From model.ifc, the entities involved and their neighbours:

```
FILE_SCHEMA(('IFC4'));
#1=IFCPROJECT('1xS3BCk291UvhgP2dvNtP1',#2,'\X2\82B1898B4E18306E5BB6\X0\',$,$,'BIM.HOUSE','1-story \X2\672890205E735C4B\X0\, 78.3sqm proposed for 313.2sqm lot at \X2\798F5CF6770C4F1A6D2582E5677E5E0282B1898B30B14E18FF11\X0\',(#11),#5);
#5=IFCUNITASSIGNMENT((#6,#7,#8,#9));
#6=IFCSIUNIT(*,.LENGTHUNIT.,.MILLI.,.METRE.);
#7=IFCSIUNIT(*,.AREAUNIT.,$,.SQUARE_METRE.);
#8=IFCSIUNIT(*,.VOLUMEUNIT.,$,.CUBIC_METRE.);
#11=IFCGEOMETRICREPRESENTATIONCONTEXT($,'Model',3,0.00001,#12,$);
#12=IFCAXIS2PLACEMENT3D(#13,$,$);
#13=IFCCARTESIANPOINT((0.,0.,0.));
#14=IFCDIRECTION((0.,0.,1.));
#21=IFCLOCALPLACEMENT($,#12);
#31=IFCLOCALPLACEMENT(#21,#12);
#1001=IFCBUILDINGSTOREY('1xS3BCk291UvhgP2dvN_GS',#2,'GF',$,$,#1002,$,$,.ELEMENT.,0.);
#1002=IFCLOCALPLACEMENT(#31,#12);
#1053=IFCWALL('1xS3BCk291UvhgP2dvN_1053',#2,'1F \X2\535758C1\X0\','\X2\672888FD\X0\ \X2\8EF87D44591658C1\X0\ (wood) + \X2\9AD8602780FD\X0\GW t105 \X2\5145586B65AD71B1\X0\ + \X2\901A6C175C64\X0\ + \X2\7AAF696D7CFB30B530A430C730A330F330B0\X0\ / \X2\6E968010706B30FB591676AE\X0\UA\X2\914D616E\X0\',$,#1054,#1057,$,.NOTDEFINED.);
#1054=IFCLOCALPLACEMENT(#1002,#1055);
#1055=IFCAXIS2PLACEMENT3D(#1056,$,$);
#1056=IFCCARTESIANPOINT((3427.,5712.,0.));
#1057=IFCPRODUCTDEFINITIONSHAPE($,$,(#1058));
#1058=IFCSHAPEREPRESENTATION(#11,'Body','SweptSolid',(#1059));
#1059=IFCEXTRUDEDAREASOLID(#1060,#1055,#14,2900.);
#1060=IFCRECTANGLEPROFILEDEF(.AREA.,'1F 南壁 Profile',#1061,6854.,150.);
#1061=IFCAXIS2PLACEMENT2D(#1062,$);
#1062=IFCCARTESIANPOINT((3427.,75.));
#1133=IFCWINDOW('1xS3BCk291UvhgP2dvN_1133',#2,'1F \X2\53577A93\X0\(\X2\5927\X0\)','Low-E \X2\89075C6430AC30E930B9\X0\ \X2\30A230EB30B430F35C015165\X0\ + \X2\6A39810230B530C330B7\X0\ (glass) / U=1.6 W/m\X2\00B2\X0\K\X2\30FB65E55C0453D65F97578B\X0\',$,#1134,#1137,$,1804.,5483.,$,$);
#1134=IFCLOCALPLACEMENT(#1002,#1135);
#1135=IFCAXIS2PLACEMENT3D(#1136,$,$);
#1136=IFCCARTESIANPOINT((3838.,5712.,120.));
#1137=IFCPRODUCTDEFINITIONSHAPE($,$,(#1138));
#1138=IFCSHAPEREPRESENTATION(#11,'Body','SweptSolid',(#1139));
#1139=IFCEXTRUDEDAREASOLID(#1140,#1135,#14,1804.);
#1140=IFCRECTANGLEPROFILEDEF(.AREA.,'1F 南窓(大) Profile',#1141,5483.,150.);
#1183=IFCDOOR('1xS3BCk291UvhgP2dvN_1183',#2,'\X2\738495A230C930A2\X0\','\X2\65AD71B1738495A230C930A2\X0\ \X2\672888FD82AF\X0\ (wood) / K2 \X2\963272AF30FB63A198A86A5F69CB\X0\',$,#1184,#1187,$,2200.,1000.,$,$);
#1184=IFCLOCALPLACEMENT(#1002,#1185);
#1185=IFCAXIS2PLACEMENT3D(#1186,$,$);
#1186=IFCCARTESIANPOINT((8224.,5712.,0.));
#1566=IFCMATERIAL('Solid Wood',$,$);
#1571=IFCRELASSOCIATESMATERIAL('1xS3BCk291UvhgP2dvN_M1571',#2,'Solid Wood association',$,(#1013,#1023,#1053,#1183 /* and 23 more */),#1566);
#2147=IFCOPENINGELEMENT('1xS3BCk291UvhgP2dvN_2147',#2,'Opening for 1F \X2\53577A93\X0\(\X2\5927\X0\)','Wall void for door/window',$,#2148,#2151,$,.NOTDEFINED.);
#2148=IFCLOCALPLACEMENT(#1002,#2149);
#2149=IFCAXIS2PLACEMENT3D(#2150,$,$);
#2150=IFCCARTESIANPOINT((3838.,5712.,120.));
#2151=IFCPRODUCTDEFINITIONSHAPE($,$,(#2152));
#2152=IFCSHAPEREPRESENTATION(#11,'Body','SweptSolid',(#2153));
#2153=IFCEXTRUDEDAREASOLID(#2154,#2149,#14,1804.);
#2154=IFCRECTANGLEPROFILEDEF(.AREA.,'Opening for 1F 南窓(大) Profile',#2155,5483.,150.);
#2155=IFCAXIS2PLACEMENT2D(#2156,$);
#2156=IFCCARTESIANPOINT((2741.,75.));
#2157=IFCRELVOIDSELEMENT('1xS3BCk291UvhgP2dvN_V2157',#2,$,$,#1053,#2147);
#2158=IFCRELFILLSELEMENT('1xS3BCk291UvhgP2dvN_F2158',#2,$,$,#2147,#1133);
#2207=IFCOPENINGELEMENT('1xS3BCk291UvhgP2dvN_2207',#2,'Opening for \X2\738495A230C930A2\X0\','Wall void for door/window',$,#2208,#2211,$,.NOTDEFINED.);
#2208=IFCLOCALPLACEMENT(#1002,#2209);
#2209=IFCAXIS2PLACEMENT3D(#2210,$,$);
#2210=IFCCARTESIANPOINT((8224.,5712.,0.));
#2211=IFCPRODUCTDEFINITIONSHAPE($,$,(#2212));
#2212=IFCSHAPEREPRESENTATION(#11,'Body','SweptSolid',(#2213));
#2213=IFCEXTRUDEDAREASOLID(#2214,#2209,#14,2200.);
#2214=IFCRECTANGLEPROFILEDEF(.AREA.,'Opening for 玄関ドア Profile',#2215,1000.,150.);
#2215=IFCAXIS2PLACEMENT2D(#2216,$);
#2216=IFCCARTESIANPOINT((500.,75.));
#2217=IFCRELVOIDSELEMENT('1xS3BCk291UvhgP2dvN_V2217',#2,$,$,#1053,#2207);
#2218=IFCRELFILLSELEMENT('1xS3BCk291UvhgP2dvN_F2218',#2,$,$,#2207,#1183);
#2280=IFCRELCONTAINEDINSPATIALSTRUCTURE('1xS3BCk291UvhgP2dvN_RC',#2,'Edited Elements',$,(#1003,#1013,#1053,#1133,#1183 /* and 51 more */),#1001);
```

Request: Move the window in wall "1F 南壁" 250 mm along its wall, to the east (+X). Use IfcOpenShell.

```python
import ifcopenshell
import ifcopenshell.api.geometry
import ifcopenshell.util.placement

model = ifcopenshell.open("model.ifc")

window = model.by_guid("1xS3BCk291UvhgP2dvN_1133")
opening = window.FillsVoids[0].RelatingOpeningElement
wall = opening.VoidsElements[0].RelatingBuildingElement

wall_matrix = ifcopenshell.util.placement.get_local_placement(wall.ObjectPlacement)
shift = wall_matrix[:3, 0] * 250.0
before = ifcopenshell.util.placement.get_local_placement(window.ObjectPlacement)[:3, 3].copy()

# The window is not placed relative to its opening, so move both.
for product in (opening, window):
    matrix = ifcopenshell.util.placement.get_local_placement(product.ObjectPlacement)
    matrix[:3, 3] += shift
    ifcopenshell.api.geometry.edit_object_placement(model, product=product, matrix=matrix, is_si=False)

after = ifcopenshell.util.placement.get_local_placement(window.ObjectPlacement)[:3, 3]
print("window moved by", (after - before).round(3) + 0.0)

model.write("model_edited.ifc")
```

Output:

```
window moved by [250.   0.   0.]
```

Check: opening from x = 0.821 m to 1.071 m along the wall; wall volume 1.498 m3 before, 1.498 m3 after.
